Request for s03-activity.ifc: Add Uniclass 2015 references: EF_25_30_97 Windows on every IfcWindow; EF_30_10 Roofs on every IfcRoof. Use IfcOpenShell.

First a look at what the model holds.

```python
import ifcopenshell

model = ifcopenshell.open("s03-activity.ifc")
print(model.schema)
print("classifications:", [c.Name for c in model.by_type("IfcClassification")])
for ifc_class in ("IfcDoor", "IfcRoof", "IfcStair", "IfcWall", "IfcWindow"):
    print(ifc_class, len(model.by_type(ifc_class)))
```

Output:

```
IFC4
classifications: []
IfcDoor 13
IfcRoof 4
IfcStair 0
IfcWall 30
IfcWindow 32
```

```python
import ifcopenshell
import ifcopenshell.api.classification

model = ifcopenshell.open("s03-activity.ifc")

system = ifcopenshell.api.classification.add_classification(model, classification="Uniclass 2015")

codes = {
    "IfcWindow": ("EF_25_30_97", "Windows"),
    "IfcRoof": ("EF_30_10", "Roofs"),
}
for ifc_class, (code, name) in codes.items():
    products = model.by_type(ifc_class)
    ifcopenshell.api.classification.add_reference(
        model, products=products, classification=system, identification=code, name=name
    )
    print(code, len(products))

model.write("s03-activity_edited.ifc")
```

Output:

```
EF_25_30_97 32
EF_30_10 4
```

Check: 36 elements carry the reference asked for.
